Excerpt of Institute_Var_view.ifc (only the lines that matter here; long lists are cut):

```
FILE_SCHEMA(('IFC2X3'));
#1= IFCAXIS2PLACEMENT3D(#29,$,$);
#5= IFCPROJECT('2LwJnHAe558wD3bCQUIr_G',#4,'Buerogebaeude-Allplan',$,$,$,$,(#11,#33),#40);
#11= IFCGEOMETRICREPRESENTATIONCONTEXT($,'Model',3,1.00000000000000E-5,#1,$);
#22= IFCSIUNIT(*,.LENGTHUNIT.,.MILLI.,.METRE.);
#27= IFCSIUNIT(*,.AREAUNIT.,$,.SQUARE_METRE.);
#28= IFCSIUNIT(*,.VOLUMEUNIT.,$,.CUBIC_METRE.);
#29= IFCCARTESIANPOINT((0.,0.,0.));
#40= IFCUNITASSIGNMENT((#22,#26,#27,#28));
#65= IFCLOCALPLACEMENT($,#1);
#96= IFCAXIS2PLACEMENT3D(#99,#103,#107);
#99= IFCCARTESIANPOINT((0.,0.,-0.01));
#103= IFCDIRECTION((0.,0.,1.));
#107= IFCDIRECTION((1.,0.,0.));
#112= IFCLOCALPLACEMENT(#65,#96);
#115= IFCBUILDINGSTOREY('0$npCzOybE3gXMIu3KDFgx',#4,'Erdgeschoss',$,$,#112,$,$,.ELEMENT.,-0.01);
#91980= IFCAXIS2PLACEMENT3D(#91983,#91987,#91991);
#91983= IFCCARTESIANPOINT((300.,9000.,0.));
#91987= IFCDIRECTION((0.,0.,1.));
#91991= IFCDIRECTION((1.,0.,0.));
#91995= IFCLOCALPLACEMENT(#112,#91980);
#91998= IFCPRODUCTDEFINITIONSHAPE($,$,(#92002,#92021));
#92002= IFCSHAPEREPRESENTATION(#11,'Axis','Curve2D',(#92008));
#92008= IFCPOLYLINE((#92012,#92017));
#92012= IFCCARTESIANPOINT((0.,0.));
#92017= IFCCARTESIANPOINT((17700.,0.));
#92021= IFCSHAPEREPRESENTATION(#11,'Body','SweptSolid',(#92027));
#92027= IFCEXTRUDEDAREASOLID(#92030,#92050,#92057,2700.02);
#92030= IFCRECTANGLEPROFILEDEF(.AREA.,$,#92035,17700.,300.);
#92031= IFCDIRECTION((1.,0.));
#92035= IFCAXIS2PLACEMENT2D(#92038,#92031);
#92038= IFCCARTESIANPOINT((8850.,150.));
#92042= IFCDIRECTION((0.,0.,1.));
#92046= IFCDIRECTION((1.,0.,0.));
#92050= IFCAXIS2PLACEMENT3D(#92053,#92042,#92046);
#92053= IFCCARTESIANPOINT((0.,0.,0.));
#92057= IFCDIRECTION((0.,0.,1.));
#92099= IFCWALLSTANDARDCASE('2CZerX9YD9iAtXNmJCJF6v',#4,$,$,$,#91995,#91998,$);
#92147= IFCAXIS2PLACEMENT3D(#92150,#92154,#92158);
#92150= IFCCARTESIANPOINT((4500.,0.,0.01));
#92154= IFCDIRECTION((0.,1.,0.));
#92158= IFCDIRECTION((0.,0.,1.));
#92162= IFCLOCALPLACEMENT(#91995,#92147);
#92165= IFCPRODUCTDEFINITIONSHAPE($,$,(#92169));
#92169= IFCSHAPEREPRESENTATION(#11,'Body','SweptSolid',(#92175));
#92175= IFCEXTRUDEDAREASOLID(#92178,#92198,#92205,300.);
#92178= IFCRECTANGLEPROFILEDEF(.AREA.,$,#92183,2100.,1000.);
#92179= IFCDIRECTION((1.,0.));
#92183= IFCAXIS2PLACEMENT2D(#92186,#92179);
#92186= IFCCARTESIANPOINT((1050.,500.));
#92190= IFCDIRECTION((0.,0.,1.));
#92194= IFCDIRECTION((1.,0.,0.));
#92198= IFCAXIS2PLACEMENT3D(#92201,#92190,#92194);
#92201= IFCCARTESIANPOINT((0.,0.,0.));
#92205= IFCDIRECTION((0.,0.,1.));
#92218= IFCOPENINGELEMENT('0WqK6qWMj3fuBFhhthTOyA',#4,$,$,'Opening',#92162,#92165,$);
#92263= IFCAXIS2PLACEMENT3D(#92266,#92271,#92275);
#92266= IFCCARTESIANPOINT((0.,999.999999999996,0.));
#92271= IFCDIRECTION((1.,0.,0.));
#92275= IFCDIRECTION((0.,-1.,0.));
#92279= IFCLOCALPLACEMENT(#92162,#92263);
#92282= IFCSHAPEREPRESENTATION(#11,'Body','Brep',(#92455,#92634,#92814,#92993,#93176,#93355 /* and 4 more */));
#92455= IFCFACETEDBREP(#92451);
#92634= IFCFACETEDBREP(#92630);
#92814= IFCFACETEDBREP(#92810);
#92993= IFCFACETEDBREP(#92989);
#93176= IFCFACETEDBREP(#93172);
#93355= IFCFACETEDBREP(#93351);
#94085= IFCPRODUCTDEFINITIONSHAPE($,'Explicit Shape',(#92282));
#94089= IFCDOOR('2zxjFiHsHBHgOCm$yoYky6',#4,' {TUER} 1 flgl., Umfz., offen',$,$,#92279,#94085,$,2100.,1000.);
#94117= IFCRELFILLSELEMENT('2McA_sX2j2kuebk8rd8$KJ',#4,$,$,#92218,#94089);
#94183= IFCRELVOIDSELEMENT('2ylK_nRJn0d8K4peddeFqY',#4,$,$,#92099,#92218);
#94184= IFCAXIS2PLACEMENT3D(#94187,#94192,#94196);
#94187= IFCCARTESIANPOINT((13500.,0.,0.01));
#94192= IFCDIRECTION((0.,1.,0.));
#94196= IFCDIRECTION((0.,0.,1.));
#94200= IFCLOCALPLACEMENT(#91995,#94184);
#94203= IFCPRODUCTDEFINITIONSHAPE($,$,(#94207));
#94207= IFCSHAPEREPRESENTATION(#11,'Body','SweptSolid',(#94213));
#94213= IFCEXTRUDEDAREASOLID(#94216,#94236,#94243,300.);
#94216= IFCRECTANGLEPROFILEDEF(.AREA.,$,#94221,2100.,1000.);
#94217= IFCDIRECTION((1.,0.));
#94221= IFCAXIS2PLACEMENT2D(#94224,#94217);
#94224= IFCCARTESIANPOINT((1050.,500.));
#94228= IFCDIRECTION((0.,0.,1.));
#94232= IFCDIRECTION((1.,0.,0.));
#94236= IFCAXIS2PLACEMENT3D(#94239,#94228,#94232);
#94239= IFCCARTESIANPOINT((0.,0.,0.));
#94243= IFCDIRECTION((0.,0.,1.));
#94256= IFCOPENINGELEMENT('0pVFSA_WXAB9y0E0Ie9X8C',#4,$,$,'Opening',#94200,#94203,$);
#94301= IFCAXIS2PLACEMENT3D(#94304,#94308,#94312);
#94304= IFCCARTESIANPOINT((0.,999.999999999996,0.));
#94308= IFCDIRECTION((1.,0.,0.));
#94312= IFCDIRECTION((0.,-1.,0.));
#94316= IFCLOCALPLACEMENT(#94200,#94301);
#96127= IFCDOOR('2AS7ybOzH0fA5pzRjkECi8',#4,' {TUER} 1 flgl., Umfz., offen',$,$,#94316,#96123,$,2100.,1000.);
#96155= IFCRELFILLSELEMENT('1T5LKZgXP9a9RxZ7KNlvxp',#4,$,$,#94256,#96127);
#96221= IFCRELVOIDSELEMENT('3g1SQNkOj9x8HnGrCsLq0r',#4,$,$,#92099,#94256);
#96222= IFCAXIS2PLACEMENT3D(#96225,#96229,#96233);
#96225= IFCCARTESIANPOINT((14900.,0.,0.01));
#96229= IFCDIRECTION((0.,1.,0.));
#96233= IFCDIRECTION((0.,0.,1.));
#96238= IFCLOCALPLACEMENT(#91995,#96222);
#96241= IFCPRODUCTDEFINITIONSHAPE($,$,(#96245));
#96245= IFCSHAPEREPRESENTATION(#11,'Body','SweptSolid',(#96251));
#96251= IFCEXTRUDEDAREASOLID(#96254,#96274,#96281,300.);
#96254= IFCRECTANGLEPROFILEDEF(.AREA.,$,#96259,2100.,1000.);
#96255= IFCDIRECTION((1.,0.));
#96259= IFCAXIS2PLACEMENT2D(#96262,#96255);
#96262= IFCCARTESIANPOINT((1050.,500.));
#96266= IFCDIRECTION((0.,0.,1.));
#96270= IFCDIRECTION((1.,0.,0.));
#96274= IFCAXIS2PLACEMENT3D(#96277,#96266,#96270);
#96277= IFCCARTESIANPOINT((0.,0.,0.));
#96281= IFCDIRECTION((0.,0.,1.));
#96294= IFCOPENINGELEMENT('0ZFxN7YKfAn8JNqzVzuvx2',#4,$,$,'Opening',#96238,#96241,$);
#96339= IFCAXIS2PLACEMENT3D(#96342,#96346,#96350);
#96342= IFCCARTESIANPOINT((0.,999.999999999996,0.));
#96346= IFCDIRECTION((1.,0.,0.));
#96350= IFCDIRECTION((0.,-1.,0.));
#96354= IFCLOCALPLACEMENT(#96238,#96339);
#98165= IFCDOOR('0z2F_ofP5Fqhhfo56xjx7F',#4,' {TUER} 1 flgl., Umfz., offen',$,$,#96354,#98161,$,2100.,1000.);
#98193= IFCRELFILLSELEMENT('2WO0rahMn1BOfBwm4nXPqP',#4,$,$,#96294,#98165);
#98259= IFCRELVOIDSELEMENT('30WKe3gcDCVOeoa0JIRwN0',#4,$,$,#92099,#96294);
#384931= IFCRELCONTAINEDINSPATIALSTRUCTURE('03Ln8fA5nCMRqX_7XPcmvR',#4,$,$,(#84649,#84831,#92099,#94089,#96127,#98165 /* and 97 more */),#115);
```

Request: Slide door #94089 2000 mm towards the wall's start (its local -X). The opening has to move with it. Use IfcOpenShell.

```python
import ifcopenshell
import ifcopenshell.api.geometry
import ifcopenshell.util.placement
import ifcopenshell.util.unit

model = ifcopenshell.open("Institute_Var_view.ifc")
unit_scale = ifcopenshell.util.unit.calculate_unit_scale(model)

door = model.by_guid("2zxjFiHsHBHgOCm$yoYky6")
opening = door.FillsVoids[0].RelatingOpeningElement
wall = opening.VoidsElements[0].RelatingBuildingElement

wall_matrix = ifcopenshell.util.placement.get_local_placement(wall.ObjectPlacement)
shift = wall_matrix[:3, 0] * -2 / unit_scale
before = ifcopenshell.util.placement.get_local_placement(door.ObjectPlacement)[:3, 3].copy()

# The door is placed relative to its opening, so it follows when the opening moves.
matrix = ifcopenshell.util.placement.get_local_placement(opening.ObjectPlacement)
matrix[:3, 3] += shift
ifcopenshell.api.geometry.edit_object_placement(
    model, product=opening, matrix=matrix, is_si=False, should_transform_children=True
)

after = ifcopenshell.util.placement.get_local_placement(door.ObjectPlacement)[:3, 3]
print("door moved by", (after - before).round(3) + 0.0)

model.write("Institute_Var_view_edited.ifc")
```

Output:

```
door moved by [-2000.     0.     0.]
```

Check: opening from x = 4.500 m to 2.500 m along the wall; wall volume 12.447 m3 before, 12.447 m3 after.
